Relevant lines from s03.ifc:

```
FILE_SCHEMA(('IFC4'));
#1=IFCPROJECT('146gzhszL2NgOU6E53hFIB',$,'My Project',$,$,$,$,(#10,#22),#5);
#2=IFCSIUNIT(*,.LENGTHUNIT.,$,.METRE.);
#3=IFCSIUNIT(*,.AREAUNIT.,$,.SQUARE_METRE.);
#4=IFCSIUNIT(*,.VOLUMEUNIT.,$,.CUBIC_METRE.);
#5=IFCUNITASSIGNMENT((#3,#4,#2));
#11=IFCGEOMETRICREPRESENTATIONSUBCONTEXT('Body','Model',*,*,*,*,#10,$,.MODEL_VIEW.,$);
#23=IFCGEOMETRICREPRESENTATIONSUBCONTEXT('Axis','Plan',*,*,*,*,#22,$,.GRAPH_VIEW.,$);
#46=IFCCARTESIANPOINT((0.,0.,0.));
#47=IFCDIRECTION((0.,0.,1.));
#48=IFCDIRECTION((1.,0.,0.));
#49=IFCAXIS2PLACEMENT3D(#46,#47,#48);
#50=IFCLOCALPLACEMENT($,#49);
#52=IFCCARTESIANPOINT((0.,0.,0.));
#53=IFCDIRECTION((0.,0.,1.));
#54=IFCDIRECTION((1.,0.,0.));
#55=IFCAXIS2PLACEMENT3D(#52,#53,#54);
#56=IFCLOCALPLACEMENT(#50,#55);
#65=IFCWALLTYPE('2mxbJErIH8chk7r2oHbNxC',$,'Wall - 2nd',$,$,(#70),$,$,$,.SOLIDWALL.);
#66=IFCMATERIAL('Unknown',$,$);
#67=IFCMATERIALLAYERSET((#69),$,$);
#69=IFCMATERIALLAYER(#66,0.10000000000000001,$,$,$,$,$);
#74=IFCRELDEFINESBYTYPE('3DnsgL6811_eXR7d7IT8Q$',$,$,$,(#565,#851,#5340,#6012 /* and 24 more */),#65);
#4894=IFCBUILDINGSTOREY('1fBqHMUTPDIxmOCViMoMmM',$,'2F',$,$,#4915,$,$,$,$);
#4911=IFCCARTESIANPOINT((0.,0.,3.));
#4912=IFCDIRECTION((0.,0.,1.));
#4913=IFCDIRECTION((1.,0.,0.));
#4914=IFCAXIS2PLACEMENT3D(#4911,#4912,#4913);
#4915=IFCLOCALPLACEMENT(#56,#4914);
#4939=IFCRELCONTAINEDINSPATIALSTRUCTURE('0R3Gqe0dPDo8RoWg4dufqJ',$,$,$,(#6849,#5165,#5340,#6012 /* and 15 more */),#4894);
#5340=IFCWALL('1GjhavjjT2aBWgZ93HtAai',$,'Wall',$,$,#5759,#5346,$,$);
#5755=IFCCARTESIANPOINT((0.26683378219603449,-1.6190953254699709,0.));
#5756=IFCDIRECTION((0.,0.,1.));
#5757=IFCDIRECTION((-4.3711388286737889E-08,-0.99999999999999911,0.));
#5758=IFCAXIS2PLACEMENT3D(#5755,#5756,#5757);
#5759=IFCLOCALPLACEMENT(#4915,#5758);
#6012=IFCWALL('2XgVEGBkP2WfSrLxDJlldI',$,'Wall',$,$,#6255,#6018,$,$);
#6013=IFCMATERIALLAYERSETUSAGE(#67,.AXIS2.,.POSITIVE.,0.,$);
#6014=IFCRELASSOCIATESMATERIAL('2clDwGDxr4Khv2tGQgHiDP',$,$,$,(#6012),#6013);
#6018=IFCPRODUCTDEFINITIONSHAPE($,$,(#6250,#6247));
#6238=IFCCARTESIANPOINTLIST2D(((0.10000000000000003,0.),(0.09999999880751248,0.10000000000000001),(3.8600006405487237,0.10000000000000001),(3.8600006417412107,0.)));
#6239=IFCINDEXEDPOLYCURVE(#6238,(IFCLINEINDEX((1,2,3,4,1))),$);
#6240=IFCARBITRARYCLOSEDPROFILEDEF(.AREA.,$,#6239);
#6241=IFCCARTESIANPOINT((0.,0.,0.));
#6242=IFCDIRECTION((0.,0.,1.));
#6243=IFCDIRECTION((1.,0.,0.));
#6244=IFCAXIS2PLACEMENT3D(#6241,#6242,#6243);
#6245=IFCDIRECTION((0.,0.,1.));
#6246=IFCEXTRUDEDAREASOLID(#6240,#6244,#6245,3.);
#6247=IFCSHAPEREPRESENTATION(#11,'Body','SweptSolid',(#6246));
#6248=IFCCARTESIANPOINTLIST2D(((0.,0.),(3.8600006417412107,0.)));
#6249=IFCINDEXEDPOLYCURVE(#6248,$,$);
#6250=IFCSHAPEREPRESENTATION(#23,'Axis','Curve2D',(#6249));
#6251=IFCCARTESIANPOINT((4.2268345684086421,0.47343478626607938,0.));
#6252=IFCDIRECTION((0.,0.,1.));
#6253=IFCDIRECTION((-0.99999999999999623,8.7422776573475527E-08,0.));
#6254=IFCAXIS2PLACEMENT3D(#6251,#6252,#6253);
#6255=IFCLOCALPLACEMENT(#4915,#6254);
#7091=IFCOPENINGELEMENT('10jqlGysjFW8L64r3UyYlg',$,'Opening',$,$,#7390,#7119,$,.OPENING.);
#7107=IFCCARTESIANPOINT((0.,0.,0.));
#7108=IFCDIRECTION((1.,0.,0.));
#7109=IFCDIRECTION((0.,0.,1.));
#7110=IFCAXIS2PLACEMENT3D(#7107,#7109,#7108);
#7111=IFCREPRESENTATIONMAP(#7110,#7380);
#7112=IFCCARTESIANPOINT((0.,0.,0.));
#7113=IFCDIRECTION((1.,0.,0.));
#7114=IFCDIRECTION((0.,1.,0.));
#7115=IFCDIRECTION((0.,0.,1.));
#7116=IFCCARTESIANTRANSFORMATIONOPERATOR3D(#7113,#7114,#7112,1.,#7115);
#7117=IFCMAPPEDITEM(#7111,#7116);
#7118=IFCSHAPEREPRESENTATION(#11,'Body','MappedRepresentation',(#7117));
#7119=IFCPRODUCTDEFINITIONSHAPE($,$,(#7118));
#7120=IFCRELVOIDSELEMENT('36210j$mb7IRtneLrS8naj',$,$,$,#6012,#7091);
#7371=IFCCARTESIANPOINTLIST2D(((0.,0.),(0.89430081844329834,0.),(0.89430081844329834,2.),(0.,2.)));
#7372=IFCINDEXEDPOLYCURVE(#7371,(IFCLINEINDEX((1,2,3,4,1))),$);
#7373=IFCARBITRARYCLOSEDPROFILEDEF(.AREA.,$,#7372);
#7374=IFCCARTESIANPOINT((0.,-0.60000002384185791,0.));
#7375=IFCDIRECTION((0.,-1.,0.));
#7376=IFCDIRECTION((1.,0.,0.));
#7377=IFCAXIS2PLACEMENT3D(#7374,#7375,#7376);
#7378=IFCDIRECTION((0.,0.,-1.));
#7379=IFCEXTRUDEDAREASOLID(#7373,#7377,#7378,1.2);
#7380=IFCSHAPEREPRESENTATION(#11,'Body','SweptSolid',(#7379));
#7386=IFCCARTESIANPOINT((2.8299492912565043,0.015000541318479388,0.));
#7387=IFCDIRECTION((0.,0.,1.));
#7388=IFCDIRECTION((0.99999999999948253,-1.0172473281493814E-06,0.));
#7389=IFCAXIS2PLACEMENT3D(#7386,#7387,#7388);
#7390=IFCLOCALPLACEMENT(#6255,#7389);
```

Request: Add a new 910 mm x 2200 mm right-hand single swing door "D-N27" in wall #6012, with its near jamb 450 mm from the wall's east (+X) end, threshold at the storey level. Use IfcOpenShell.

```python
import numpy as np
import ifcopenshell
import ifcopenshell.api.feature
import ifcopenshell.api.geometry
import ifcopenshell.api.root
import ifcopenshell.api.spatial
import ifcopenshell.geom
import ifcopenshell.util.element
import ifcopenshell.util.placement
import ifcopenshell.util.representation
import ifcopenshell.util.shape
import ifcopenshell.util.unit

model = ifcopenshell.open("s03.ifc")
unit_scale = ifcopenshell.util.unit.calculate_unit_scale(model)
settings = ifcopenshell.geom.settings()


def volume(element):
    """Net volume in cubic metres, openings subtracted."""
    shape = ifcopenshell.geom.create_shape(settings, element)
    return ifcopenshell.util.shape.get_volume(shape.geometry)


wall = model.by_id(6012)
storey = ifcopenshell.util.element.get_container(wall, ifc_class="IfcBuildingStorey")
context = ifcopenshell.util.representation.get_context(model, "Model", "Body", "MODEL_VIEW")
before = volume(wall)

width, height, from_end, sill = 0.91, 2.2, 0.45, 0.0  # metres

# The wall runs along its own X axis, and the end named is its -X end.
wall_shape = ifcopenshell.geom.create_shape(settings, wall)
x, y, z = ifcopenshell.util.shape.get_vertices(wall_shape.geometry).T
start = x.min() + from_end
face, thickness = float(y.min()), float(y.max() - y.min())
wall_matrix = ifcopenshell.util.placement.get_local_placement(wall.ObjectPlacement)
level = ifcopenshell.util.placement.get_local_placement(storey.ObjectPlacement)[2, 3]


def in_wall(x, y):
    """Placement at x, y metres in the wall's axes, at sill height."""
    matrix = wall_matrix.copy()
    matrix[:, 3] = wall_matrix @ np.array([x / unit_scale, y / unit_scale, 0.0, 1.0])
    matrix[2, 3] = level + sill / unit_scale
    return matrix


# Opening: a box that overshoots both wall faces by 50 mm.
opening = ifcopenshell.api.root.create_entity(model, ifc_class="IfcOpeningElement", predefined_type="OPENING")
box = ifcopenshell.api.geometry.add_wall_representation(
    model, context=context, length=width, height=height, thickness=thickness + 0.1
)
ifcopenshell.api.geometry.assign_representation(model, product=opening, representation=box)
ifcopenshell.api.geometry.edit_object_placement(model, product=opening, matrix=in_wall(start, face - 0.05), is_si=False)
ifcopenshell.api.feature.add_feature(model, feature=opening, element=wall)

door = ifcopenshell.api.root.create_entity(model, ifc_class="IfcDoor", name="D-N27", predefined_type="DOOR")
door.OverallWidth, door.OverallHeight = width / unit_scale, height / unit_scale
door.OperationType = "SINGLE_SWING_RIGHT"
body = ifcopenshell.api.geometry.add_door_representation(
    model,
    context=context,
    overall_width=door.OverallWidth,
    overall_height=door.OverallHeight,
    operation_type="SINGLE_SWING_RIGHT",
    lining_properties={"LiningDepth": thickness / unit_scale, "ThresholdDepth": thickness / unit_scale},
)
ifcopenshell.api.geometry.assign_representation(model, product=door, representation=body)
ifcopenshell.api.spatial.assign_container(model, products=[door], relating_structure=storey)
ifcopenshell.api.feature.add_filling(model, opening=opening, element=door)

# The lining spans the wall, so the door starts at the wall face.
ifcopenshell.api.geometry.edit_object_placement(model, product=door, matrix=in_wall(start, face), is_si=False)

after = volume(wall)

print(f"wall volume {before:.3f} -> {after:.3f} m3")

model.write("s03-out.ifc")
```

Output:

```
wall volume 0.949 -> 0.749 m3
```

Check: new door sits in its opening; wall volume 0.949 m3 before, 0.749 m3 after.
